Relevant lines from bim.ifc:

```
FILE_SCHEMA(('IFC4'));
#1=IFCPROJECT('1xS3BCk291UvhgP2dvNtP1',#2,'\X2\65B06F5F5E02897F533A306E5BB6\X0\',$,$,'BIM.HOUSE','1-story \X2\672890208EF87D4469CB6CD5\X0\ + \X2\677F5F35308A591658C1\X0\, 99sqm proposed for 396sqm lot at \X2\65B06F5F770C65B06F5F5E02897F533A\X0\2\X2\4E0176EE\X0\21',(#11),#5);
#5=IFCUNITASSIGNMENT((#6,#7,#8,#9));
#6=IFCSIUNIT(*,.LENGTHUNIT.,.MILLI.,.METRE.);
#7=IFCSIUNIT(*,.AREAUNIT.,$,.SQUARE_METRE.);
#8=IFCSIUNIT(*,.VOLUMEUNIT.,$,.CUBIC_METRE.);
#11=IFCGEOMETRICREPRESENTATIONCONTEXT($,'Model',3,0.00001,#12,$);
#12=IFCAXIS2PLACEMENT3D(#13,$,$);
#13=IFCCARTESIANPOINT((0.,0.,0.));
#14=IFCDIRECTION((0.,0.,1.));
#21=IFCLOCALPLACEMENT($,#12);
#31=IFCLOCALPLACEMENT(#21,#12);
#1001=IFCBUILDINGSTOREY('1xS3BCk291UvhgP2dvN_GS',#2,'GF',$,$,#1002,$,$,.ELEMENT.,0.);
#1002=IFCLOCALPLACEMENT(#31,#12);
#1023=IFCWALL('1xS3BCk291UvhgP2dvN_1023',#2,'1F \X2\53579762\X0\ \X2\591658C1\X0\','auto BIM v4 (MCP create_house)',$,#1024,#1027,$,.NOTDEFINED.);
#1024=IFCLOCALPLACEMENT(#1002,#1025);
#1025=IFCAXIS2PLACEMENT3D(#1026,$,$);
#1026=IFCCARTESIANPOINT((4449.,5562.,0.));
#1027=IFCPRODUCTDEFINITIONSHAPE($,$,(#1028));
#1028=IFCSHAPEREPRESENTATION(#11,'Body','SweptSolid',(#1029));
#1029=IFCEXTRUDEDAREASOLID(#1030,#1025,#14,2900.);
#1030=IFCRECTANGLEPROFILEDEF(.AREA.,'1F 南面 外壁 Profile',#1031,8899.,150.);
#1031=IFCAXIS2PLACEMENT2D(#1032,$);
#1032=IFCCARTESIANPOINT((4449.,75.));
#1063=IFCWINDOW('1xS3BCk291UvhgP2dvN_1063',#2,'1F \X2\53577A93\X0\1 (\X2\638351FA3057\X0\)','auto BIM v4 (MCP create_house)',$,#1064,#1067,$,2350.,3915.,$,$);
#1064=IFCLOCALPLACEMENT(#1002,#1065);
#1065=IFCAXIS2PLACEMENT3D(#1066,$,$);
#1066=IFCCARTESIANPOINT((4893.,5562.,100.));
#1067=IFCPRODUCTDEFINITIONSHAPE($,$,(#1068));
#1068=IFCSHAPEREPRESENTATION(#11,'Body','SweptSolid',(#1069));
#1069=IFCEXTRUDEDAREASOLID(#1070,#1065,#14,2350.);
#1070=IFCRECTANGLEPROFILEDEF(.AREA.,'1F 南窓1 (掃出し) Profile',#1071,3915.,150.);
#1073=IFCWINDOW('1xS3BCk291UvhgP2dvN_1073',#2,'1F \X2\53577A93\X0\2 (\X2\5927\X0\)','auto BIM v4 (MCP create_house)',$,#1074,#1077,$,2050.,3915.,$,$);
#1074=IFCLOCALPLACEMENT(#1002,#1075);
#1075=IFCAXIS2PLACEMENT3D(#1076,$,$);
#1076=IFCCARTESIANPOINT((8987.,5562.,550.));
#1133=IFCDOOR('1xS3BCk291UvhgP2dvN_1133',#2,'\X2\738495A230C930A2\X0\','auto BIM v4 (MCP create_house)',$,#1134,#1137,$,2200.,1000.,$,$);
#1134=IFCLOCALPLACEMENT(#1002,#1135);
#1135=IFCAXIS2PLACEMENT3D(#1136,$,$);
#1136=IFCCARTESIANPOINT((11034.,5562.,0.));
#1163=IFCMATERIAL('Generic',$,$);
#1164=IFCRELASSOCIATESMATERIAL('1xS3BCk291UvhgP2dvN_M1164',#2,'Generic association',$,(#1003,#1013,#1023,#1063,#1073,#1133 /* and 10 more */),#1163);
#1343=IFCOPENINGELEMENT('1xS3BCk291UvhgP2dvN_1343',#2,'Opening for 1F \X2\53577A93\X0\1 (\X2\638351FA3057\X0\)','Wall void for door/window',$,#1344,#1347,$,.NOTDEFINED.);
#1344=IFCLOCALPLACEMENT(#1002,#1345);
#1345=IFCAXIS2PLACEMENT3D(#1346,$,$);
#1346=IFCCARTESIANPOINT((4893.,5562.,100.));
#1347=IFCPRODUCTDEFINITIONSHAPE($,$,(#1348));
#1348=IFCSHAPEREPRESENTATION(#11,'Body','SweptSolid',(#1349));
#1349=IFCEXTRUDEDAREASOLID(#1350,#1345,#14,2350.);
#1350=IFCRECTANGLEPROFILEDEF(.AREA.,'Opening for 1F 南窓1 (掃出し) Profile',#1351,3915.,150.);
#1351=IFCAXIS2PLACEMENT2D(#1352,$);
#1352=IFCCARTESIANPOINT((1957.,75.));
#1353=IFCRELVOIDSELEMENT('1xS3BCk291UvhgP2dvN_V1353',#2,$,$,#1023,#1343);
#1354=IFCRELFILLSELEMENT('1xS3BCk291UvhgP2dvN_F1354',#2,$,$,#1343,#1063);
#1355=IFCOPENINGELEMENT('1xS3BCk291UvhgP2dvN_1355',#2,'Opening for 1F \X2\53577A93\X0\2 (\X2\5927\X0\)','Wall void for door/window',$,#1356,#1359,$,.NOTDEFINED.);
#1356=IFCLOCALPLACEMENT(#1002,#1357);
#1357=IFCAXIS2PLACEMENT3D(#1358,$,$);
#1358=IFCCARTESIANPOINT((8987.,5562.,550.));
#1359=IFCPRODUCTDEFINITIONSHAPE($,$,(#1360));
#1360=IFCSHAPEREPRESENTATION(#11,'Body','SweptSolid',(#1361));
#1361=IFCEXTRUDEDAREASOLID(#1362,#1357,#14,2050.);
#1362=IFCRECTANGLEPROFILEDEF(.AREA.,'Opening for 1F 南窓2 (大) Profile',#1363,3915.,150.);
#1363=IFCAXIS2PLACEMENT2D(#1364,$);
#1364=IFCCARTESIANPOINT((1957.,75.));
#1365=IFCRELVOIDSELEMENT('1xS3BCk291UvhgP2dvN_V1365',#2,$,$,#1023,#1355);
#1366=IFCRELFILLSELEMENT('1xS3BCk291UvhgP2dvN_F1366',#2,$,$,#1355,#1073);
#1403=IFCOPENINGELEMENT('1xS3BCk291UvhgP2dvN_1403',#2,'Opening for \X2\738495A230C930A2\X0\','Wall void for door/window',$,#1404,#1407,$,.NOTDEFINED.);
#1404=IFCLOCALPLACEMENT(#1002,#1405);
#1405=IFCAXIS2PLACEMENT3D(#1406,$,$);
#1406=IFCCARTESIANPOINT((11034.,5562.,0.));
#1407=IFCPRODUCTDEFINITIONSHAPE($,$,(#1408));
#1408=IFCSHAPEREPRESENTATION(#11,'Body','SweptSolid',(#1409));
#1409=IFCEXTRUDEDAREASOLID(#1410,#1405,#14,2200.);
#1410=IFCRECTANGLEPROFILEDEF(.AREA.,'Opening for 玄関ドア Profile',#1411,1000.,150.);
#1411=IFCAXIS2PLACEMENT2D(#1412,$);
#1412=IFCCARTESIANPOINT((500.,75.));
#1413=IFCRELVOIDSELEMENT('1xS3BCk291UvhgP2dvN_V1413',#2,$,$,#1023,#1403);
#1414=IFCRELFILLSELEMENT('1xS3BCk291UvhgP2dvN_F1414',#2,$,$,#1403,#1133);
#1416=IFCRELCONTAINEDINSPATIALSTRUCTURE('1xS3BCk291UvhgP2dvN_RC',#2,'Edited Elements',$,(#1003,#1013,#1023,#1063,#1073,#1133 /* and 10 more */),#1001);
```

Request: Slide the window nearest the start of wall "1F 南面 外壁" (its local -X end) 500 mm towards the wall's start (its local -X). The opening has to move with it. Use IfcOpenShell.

```python
import ifcopenshell
import ifcopenshell.api.geometry
import ifcopenshell.util.placement
import ifcopenshell.util.unit

model = ifcopenshell.open("bim.ifc")
unit_scale = ifcopenshell.util.unit.calculate_unit_scale(model)

window = model.by_guid("1xS3BCk291UvhgP2dvN_1063")
opening = window.FillsVoids[0].RelatingOpeningElement
wall = opening.VoidsElements[0].RelatingBuildingElement

wall_matrix = ifcopenshell.util.placement.get_local_placement(wall.ObjectPlacement)
shift = wall_matrix[:3, 0] * -0.5 / unit_scale
before = ifcopenshell.util.placement.get_local_placement(window.ObjectPlacement)[:3, 3].copy()

# The window is not placed relative to its opening, so move both.
for product in (opening, window):
    matrix = ifcopenshell.util.placement.get_local_placement(product.ObjectPlacement)
    matrix[:3, 3] += shift
    ifcopenshell.api.geometry.edit_object_placement(model, product=product, matrix=matrix, is_si=False)

after = ifcopenshell.util.placement.get_local_placement(window.ObjectPlacement)[:3, 3]
print("window moved by", (after - before).round(3) + 0.0)

model.write("bim_rev.ifc")
```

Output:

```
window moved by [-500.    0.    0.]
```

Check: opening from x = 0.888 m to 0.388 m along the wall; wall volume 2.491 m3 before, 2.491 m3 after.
